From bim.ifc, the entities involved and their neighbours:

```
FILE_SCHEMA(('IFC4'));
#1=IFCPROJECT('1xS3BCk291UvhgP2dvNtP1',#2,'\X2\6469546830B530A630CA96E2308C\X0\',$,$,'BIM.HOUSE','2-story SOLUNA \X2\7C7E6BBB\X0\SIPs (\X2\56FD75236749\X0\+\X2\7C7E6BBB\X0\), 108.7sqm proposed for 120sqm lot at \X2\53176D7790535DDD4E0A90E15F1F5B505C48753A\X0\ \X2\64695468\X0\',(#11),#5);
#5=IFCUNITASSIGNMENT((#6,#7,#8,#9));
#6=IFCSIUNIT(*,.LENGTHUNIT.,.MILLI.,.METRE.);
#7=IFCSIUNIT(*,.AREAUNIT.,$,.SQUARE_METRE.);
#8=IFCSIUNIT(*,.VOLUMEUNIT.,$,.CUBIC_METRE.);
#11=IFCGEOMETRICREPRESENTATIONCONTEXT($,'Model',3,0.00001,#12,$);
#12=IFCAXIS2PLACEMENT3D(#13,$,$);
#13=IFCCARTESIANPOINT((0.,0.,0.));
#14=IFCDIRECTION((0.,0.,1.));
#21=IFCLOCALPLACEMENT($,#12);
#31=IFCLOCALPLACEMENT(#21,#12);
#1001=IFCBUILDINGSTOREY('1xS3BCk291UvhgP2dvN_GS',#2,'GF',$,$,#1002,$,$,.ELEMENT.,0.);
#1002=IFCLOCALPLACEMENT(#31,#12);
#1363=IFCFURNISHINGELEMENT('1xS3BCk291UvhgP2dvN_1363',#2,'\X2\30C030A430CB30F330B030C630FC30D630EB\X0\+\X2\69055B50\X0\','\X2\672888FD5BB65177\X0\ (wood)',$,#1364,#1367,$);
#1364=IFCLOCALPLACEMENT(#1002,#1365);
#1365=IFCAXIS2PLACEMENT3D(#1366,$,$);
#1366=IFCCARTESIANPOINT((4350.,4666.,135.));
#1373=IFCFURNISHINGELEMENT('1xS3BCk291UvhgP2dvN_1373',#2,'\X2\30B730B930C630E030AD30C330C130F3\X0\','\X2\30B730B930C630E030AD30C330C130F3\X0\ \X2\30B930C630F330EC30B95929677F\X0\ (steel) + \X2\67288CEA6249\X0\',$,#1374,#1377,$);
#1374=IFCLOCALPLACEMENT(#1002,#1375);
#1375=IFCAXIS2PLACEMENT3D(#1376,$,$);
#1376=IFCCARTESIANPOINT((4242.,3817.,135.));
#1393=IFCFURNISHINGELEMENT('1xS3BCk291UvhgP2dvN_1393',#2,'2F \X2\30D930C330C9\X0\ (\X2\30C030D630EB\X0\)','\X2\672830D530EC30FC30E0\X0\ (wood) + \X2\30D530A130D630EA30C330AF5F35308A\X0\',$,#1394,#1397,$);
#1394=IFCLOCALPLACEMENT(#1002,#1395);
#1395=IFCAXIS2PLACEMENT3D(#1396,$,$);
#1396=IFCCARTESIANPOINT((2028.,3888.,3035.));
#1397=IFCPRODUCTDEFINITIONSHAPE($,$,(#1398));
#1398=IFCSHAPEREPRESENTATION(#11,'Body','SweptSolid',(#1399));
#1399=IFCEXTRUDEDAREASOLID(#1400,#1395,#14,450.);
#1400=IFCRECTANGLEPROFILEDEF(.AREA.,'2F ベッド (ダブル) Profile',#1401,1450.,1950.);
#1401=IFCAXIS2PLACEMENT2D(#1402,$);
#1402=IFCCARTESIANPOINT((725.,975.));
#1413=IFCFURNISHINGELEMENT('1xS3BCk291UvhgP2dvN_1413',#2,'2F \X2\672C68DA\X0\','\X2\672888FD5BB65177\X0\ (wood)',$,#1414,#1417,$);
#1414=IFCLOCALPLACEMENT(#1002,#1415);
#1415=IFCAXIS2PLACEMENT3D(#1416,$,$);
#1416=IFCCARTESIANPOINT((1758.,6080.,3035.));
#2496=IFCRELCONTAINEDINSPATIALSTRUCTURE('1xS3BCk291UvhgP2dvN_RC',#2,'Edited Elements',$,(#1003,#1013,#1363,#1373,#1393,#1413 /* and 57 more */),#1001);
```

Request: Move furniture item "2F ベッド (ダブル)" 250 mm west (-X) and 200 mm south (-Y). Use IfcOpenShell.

```python
import ifcopenshell
import ifcopenshell.api.geometry
import ifcopenshell.util.placement

model = ifcopenshell.open("bim.ifc")

item = model.by_id(1393)
matrix = ifcopenshell.util.placement.get_local_placement(item.ObjectPlacement)
matrix[0, 3] -= 250.0
matrix[1, 3] -= 200.0
ifcopenshell.api.geometry.edit_object_placement(model, product=item, matrix=matrix, is_si=False)

print(ifcopenshell.util.placement.get_local_placement(item.ObjectPlacement).round(3) + 0.0)

model.write("bim_updated.ifc")
```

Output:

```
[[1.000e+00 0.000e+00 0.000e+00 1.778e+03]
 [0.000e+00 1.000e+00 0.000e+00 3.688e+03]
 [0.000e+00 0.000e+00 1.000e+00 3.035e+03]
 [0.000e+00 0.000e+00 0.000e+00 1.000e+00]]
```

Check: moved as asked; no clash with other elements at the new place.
